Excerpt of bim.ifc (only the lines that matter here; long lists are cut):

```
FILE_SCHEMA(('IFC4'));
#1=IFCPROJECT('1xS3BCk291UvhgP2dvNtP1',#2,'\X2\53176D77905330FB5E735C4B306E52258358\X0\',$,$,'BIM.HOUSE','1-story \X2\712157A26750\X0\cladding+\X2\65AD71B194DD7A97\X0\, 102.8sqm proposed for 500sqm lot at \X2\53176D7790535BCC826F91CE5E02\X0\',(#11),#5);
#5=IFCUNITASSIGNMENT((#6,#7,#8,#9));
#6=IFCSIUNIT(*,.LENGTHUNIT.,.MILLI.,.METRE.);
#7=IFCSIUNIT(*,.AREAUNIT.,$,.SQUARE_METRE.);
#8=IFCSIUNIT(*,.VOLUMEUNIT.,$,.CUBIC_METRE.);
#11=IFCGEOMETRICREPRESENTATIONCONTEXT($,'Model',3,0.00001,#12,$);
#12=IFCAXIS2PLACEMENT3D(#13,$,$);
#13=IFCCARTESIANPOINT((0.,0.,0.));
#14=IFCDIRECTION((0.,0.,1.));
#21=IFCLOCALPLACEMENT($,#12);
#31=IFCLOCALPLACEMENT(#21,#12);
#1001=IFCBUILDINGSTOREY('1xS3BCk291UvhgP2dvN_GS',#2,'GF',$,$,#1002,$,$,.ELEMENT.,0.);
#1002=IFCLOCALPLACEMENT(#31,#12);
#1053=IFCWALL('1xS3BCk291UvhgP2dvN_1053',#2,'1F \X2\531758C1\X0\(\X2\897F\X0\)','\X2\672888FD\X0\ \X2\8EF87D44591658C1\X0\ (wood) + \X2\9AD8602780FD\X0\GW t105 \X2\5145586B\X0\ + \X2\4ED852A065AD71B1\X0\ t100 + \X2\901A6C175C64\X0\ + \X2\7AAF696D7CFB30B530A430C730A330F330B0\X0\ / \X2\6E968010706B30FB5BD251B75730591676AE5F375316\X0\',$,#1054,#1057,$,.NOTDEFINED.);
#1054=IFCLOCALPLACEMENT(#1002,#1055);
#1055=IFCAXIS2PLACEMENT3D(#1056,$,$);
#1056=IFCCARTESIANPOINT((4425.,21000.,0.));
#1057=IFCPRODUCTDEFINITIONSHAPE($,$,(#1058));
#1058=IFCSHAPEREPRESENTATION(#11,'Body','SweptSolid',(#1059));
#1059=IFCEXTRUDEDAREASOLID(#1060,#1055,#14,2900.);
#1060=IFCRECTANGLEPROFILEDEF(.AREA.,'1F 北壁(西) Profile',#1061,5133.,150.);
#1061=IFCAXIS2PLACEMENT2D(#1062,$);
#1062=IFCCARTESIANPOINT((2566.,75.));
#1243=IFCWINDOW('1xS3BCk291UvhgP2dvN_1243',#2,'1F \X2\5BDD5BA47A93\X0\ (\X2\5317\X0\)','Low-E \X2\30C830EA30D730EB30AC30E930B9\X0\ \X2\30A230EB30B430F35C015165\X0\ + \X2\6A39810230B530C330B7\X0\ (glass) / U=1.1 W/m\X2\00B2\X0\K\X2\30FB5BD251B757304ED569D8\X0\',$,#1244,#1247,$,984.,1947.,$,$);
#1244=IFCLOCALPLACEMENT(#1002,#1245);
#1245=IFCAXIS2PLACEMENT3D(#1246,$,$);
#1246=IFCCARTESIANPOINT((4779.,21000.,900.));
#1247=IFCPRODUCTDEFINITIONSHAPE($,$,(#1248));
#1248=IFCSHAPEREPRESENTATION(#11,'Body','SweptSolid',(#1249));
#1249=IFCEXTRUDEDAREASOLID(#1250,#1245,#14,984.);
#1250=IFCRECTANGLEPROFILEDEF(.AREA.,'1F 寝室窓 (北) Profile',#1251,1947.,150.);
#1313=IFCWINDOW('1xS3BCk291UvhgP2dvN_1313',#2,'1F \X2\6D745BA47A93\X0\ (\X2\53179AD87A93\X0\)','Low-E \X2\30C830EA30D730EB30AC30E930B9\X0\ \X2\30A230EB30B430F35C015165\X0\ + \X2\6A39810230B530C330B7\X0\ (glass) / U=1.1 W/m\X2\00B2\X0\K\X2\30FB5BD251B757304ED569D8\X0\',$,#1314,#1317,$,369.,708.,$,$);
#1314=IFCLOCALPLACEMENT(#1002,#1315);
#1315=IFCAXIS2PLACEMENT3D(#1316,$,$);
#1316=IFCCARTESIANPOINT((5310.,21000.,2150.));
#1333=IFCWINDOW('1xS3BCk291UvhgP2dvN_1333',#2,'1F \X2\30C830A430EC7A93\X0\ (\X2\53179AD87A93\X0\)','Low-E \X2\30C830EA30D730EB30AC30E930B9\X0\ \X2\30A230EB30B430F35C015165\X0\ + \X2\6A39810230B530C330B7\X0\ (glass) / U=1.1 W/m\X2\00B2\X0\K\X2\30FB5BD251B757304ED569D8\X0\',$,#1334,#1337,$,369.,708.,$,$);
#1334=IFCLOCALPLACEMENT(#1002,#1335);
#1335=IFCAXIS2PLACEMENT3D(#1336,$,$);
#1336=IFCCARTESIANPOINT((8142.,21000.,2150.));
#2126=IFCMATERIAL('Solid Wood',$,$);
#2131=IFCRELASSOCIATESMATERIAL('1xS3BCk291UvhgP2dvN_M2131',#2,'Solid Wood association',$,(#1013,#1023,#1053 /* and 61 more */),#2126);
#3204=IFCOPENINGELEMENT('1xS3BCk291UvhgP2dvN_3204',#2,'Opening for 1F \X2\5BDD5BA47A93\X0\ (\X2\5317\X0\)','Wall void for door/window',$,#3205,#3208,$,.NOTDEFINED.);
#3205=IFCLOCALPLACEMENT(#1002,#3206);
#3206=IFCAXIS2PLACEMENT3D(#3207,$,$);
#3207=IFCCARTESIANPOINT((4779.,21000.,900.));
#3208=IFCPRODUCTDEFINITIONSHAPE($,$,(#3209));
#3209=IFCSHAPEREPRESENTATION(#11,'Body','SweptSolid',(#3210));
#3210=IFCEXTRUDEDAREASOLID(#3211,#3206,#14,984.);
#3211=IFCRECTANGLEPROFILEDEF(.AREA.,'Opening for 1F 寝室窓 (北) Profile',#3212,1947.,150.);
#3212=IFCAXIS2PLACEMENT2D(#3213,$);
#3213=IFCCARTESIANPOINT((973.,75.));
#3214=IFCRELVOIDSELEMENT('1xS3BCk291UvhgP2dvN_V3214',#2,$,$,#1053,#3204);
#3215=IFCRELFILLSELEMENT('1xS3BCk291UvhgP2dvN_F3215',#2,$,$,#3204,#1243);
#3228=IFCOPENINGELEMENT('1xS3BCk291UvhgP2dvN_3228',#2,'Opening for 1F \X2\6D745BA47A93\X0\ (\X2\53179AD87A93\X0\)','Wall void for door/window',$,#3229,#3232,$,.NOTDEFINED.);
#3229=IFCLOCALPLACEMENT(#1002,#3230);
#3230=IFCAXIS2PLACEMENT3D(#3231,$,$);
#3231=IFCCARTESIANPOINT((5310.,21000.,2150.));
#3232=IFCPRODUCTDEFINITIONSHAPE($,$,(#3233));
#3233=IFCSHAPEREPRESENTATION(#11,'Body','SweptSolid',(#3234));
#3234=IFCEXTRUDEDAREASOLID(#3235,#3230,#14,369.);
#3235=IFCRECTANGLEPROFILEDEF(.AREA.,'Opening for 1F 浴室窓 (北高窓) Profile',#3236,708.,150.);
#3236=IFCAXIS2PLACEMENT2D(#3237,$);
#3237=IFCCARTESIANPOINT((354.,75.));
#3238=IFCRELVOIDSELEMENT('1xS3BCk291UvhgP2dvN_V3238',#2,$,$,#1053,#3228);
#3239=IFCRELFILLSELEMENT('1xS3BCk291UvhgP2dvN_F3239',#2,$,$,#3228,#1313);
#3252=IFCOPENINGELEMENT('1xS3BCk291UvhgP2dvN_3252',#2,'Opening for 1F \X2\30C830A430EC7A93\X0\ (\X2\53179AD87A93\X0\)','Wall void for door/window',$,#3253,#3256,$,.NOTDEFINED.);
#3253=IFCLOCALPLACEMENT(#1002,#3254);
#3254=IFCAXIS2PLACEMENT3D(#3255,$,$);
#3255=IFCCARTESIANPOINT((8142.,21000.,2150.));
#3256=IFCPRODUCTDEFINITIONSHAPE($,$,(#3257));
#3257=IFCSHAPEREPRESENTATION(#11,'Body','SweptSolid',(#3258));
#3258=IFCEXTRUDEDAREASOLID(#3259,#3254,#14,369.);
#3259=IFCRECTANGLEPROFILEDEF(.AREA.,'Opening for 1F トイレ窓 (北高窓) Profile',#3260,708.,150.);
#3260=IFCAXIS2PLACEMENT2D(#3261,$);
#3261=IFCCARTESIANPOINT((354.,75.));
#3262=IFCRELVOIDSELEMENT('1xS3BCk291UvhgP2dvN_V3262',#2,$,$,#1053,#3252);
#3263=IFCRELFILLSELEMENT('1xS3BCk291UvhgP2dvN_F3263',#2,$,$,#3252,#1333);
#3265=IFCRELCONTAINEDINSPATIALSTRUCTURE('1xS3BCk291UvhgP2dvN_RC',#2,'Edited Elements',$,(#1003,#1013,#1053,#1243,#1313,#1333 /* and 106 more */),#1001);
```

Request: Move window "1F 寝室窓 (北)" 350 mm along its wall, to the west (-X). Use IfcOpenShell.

```python
import ifcopenshell
import ifcopenshell.api.geometry
import ifcopenshell.util.placement
import ifcopenshell.util.unit

model = ifcopenshell.open("bim.ifc")
unit_scale = ifcopenshell.util.unit.calculate_unit_scale(model)

window = model.by_guid("1xS3BCk291UvhgP2dvN_1243")
opening = window.FillsVoids[0].RelatingOpeningElement
wall = opening.VoidsElements[0].RelatingBuildingElement

wall_matrix = ifcopenshell.util.placement.get_local_placement(wall.ObjectPlacement)
shift = wall_matrix[:3, 0] * -0.35 / unit_scale
before = ifcopenshell.util.placement.get_local_placement(window.ObjectPlacement)[:3, 3].copy()

# The window is not placed relative to its opening, so move both.
for product in (opening, window):
    matrix = ifcopenshell.util.placement.get_local_placement(product.ObjectPlacement)
    matrix[:3, 3] += shift
    ifcopenshell.api.geometry.edit_object_placement(model, product=product, matrix=matrix, is_si=False)

after = ifcopenshell.util.placement.get_local_placement(window.ObjectPlacement)[:3, 3]
print("window moved by", (after - before).round(3) + 0.0)

model.write("bim_rev.ifc")
```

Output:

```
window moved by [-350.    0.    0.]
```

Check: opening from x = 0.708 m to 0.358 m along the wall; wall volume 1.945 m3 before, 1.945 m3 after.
